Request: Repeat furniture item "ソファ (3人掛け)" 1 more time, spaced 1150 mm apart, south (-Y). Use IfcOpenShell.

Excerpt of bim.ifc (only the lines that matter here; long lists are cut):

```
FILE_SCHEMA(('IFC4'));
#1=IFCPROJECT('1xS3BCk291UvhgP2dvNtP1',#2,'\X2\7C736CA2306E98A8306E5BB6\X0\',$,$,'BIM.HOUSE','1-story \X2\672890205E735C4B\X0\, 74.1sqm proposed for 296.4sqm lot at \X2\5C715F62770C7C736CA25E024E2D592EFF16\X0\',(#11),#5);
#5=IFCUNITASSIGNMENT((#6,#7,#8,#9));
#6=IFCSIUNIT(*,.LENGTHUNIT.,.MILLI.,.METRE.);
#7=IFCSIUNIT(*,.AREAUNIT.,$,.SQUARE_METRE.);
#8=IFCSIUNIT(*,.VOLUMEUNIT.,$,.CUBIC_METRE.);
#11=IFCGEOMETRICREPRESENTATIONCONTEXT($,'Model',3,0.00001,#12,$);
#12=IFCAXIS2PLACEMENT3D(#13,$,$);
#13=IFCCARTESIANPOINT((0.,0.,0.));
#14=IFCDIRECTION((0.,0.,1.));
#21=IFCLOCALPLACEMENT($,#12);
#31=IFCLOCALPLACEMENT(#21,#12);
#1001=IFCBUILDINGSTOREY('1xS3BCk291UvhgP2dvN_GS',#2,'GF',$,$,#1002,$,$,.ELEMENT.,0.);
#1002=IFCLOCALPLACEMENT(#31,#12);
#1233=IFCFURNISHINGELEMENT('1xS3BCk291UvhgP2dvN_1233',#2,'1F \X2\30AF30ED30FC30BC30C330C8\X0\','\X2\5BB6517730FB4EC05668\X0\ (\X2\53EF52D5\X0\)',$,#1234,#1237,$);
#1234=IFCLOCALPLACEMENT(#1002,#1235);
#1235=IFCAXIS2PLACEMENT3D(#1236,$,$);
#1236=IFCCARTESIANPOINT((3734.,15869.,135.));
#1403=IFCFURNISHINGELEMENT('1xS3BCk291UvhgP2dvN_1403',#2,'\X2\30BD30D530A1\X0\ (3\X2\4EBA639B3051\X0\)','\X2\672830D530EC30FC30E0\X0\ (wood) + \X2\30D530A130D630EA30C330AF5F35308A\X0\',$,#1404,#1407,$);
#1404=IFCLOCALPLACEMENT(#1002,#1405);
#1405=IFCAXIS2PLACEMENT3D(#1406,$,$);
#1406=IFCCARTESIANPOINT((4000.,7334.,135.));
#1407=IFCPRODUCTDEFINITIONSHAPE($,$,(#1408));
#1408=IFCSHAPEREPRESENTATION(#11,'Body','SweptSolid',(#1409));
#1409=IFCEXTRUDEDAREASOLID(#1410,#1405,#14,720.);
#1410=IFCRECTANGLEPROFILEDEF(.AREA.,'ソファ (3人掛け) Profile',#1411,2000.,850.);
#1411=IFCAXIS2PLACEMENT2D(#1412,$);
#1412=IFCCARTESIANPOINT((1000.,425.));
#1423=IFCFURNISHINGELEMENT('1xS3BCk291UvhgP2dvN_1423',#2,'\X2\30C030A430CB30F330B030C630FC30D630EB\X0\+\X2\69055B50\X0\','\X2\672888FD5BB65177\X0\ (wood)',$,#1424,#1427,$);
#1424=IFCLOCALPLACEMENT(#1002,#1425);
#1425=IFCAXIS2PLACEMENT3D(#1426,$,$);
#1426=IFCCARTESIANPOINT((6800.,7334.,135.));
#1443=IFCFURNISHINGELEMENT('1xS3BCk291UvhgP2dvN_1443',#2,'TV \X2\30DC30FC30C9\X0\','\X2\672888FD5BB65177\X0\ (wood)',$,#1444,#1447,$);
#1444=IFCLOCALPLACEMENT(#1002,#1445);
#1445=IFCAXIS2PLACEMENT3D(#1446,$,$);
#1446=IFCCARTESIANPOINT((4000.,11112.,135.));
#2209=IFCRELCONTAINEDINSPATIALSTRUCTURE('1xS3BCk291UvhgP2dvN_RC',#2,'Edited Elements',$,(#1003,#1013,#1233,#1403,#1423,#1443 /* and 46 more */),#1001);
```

```python
import numpy as np
import ifcopenshell
import ifcopenshell.api.geometry
import ifcopenshell.api.root
import ifcopenshell.util.element
import ifcopenshell.util.placement
import ifcopenshell.util.unit

model = ifcopenshell.open("bim.ifc")
unit_scale = ifcopenshell.util.unit.calculate_unit_scale(model)


def reuse_history(source, copy):
    """copy_class also copies each property set's owner history, people and application; keep the originals."""
    for rel in copy.IsDefinedBy:
        if rel.is_a("IfcRelDefinesByProperties") and (history := rel.RelatingPropertyDefinition.OwnerHistory):
            rel.RelatingPropertyDefinition.OwnerHistory = source.OwnerHistory
            ifcopenshell.util.element.remove_deep2(model, history)


source = model.by_guid("1xS3BCk291UvhgP2dvN_1403")
base = ifcopenshell.util.placement.get_local_placement(source.ObjectPlacement)
step = np.array([0.0, -1.0, 0.0]) * 1.15 / unit_scale

for i in range(1, 2):
    copy = ifcopenshell.api.root.copy_class(model, product=source)
    copy.Representation = ifcopenshell.util.element.copy_deep(
        model, source.Representation, exclude=["IfcGeometricRepresentationContext", "IfcRepresentationMap"]
    )
    reuse_history(source, copy)
    matrix = base.copy()
    matrix[:3, 3] += i * step
    print("added at", matrix[:3, 3].round(3) + 0.0)
    ifcopenshell.api.geometry.edit_object_placement(model, product=copy, matrix=matrix, is_si=False)

model.write("bim_v2.ifc")
```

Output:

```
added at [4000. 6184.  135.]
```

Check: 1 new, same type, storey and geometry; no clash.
